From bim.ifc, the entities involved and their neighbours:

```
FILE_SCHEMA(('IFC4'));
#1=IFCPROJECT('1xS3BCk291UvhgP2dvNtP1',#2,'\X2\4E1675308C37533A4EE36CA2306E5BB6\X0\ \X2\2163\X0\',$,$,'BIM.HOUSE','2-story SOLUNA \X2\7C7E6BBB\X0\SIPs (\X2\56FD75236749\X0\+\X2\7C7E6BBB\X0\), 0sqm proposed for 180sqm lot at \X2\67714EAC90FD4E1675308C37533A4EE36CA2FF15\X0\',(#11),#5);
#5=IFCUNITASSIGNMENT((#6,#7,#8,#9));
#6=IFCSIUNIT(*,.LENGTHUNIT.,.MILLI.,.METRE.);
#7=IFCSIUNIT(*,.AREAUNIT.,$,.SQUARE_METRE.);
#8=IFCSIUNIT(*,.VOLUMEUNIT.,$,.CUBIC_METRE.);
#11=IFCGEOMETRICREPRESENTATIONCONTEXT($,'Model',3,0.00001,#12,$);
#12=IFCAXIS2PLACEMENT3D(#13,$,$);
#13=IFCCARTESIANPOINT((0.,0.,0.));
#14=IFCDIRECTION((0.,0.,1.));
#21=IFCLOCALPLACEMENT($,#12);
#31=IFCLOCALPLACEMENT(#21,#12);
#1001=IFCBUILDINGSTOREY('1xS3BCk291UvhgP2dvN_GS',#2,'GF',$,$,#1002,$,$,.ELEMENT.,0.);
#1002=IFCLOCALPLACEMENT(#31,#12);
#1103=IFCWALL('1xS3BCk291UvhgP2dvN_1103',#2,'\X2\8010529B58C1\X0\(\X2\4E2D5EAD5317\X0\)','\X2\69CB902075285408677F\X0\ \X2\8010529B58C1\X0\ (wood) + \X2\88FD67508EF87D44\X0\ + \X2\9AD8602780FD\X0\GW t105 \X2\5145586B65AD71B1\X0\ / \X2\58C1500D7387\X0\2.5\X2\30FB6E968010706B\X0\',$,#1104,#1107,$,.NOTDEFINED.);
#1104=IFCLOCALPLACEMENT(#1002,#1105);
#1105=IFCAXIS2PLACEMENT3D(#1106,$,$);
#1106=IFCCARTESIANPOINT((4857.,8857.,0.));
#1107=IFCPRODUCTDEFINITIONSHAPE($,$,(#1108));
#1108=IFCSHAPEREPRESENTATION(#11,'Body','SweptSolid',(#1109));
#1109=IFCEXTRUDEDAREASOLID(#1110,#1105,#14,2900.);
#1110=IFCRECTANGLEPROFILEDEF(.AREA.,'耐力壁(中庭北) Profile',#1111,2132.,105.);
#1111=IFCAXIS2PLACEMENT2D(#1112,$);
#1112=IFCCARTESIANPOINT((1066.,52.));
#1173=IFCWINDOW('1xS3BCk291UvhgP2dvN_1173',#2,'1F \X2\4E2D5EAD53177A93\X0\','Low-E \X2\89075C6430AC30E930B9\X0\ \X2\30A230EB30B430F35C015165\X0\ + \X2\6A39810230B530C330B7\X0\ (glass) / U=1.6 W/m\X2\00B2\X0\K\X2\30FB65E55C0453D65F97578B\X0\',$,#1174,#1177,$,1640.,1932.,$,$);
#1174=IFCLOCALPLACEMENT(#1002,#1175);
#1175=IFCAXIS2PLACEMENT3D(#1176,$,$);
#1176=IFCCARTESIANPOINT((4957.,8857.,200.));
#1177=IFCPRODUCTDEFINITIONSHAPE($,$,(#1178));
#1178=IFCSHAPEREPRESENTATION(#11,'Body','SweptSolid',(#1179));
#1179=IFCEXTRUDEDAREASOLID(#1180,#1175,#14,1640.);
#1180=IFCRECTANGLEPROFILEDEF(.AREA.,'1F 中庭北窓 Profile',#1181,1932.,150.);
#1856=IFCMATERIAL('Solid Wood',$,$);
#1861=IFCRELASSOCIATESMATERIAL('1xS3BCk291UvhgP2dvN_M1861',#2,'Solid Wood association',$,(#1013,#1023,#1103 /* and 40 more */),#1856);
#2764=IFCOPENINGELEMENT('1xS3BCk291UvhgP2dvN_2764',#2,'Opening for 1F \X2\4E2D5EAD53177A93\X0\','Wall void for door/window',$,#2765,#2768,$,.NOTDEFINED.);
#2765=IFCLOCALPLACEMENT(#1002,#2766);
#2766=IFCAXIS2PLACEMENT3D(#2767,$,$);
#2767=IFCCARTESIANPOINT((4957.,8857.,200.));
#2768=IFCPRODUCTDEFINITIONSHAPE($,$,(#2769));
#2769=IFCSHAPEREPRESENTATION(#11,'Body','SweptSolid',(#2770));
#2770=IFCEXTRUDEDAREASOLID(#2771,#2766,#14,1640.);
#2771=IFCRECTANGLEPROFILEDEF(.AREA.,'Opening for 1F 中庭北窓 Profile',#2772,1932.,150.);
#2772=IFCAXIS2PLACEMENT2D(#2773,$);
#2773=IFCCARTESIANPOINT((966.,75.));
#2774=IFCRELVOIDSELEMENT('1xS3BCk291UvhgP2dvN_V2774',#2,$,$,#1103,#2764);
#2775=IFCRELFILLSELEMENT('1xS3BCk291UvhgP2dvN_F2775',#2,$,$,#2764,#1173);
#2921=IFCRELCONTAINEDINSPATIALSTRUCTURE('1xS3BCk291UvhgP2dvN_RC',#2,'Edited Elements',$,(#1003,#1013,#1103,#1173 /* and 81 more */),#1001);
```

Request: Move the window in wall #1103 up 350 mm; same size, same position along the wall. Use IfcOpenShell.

```python
import numpy as np
import ifcopenshell
import ifcopenshell.api.geometry
import ifcopenshell.util.placement
import ifcopenshell.util.unit

model = ifcopenshell.open("bim.ifc")
unit_scale = ifcopenshell.util.unit.calculate_unit_scale(model)

window = model.by_guid("1xS3BCk291UvhgP2dvN_1173")
opening = window.FillsVoids[0].RelatingOpeningElement
dz = 350.0

shift = np.array([0.0, 0.0, dz])
# The window is not placed relative to its opening, so move both.
for product in (opening, window):
    matrix = ifcopenshell.util.placement.get_local_placement(product.ObjectPlacement)
    matrix[:3, 3] += shift
    ifcopenshell.api.geometry.edit_object_placement(model, product=product, matrix=matrix, is_si=False)

print(f"moved by {dz * unit_scale:+.3f} m")

model.write("bim_rev.ifc")
```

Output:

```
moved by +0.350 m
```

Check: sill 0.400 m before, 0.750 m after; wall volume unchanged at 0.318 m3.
